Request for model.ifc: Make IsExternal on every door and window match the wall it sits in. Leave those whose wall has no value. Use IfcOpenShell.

First a look at what the model holds.

```python
import ifcopenshell
import ifcopenshell.util.element

model = ifcopenshell.open("model.ifc")
print(model.schema)
seen = {}
for e in model.by_type("IfcDoor") + model.by_type("IfcWindow"):
    if not e.FillsVoids:
        continue
    host = e.FillsVoids[0].RelatingOpeningElement.VoidsElements[0].RelatingBuildingElement
    own = ifcopenshell.util.element.get_pset(e, f"Pset_{e.is_a()[3:].removesuffix('StandardCase')}Common", "IsExternal")
    wall = ifcopenshell.util.element.get_pset(host, "Pset_WallCommon", "IsExternal")
    seen[e.is_a(), own, wall] = seen.get((e.is_a(), own, wall), 0) + 1
for (cls, own, wall), count in sorted(seen.items(), key=str):
    print(count, cls, "IsExternal:", own, "| host wall:", wall)
```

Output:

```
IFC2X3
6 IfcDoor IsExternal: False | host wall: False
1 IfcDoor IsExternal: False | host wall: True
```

```python
import ifcopenshell
import ifcopenshell.api.pset
import ifcopenshell.util.element

model = ifcopenshell.open("model.ifc")

count = 0
for ifc_class, pset_name in (("IfcDoor", "Pset_DoorCommon"), ("IfcWindow", "Pset_WindowCommon")):
    for e in model.by_type(ifc_class):
        if not e.FillsVoids:
            continue
        host = e.FillsVoids[0].RelatingOpeningElement.VoidsElements[0].RelatingBuildingElement
        external = ifcopenshell.util.element.get_pset(host, "Pset_WallCommon", "IsExternal")
        if external is None or ifcopenshell.util.element.get_pset(e, pset_name, "IsExternal") == external:
            continue
        pset = ifcopenshell.api.pset.add_pset(model, product=e, name=pset_name)
        ifcopenshell.api.pset.edit_pset(model, pset=pset, properties={"IsExternal": external})
        count += 1

print(count, "updated")

model.write("model_v2.ifc")
```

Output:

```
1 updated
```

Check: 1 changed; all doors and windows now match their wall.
